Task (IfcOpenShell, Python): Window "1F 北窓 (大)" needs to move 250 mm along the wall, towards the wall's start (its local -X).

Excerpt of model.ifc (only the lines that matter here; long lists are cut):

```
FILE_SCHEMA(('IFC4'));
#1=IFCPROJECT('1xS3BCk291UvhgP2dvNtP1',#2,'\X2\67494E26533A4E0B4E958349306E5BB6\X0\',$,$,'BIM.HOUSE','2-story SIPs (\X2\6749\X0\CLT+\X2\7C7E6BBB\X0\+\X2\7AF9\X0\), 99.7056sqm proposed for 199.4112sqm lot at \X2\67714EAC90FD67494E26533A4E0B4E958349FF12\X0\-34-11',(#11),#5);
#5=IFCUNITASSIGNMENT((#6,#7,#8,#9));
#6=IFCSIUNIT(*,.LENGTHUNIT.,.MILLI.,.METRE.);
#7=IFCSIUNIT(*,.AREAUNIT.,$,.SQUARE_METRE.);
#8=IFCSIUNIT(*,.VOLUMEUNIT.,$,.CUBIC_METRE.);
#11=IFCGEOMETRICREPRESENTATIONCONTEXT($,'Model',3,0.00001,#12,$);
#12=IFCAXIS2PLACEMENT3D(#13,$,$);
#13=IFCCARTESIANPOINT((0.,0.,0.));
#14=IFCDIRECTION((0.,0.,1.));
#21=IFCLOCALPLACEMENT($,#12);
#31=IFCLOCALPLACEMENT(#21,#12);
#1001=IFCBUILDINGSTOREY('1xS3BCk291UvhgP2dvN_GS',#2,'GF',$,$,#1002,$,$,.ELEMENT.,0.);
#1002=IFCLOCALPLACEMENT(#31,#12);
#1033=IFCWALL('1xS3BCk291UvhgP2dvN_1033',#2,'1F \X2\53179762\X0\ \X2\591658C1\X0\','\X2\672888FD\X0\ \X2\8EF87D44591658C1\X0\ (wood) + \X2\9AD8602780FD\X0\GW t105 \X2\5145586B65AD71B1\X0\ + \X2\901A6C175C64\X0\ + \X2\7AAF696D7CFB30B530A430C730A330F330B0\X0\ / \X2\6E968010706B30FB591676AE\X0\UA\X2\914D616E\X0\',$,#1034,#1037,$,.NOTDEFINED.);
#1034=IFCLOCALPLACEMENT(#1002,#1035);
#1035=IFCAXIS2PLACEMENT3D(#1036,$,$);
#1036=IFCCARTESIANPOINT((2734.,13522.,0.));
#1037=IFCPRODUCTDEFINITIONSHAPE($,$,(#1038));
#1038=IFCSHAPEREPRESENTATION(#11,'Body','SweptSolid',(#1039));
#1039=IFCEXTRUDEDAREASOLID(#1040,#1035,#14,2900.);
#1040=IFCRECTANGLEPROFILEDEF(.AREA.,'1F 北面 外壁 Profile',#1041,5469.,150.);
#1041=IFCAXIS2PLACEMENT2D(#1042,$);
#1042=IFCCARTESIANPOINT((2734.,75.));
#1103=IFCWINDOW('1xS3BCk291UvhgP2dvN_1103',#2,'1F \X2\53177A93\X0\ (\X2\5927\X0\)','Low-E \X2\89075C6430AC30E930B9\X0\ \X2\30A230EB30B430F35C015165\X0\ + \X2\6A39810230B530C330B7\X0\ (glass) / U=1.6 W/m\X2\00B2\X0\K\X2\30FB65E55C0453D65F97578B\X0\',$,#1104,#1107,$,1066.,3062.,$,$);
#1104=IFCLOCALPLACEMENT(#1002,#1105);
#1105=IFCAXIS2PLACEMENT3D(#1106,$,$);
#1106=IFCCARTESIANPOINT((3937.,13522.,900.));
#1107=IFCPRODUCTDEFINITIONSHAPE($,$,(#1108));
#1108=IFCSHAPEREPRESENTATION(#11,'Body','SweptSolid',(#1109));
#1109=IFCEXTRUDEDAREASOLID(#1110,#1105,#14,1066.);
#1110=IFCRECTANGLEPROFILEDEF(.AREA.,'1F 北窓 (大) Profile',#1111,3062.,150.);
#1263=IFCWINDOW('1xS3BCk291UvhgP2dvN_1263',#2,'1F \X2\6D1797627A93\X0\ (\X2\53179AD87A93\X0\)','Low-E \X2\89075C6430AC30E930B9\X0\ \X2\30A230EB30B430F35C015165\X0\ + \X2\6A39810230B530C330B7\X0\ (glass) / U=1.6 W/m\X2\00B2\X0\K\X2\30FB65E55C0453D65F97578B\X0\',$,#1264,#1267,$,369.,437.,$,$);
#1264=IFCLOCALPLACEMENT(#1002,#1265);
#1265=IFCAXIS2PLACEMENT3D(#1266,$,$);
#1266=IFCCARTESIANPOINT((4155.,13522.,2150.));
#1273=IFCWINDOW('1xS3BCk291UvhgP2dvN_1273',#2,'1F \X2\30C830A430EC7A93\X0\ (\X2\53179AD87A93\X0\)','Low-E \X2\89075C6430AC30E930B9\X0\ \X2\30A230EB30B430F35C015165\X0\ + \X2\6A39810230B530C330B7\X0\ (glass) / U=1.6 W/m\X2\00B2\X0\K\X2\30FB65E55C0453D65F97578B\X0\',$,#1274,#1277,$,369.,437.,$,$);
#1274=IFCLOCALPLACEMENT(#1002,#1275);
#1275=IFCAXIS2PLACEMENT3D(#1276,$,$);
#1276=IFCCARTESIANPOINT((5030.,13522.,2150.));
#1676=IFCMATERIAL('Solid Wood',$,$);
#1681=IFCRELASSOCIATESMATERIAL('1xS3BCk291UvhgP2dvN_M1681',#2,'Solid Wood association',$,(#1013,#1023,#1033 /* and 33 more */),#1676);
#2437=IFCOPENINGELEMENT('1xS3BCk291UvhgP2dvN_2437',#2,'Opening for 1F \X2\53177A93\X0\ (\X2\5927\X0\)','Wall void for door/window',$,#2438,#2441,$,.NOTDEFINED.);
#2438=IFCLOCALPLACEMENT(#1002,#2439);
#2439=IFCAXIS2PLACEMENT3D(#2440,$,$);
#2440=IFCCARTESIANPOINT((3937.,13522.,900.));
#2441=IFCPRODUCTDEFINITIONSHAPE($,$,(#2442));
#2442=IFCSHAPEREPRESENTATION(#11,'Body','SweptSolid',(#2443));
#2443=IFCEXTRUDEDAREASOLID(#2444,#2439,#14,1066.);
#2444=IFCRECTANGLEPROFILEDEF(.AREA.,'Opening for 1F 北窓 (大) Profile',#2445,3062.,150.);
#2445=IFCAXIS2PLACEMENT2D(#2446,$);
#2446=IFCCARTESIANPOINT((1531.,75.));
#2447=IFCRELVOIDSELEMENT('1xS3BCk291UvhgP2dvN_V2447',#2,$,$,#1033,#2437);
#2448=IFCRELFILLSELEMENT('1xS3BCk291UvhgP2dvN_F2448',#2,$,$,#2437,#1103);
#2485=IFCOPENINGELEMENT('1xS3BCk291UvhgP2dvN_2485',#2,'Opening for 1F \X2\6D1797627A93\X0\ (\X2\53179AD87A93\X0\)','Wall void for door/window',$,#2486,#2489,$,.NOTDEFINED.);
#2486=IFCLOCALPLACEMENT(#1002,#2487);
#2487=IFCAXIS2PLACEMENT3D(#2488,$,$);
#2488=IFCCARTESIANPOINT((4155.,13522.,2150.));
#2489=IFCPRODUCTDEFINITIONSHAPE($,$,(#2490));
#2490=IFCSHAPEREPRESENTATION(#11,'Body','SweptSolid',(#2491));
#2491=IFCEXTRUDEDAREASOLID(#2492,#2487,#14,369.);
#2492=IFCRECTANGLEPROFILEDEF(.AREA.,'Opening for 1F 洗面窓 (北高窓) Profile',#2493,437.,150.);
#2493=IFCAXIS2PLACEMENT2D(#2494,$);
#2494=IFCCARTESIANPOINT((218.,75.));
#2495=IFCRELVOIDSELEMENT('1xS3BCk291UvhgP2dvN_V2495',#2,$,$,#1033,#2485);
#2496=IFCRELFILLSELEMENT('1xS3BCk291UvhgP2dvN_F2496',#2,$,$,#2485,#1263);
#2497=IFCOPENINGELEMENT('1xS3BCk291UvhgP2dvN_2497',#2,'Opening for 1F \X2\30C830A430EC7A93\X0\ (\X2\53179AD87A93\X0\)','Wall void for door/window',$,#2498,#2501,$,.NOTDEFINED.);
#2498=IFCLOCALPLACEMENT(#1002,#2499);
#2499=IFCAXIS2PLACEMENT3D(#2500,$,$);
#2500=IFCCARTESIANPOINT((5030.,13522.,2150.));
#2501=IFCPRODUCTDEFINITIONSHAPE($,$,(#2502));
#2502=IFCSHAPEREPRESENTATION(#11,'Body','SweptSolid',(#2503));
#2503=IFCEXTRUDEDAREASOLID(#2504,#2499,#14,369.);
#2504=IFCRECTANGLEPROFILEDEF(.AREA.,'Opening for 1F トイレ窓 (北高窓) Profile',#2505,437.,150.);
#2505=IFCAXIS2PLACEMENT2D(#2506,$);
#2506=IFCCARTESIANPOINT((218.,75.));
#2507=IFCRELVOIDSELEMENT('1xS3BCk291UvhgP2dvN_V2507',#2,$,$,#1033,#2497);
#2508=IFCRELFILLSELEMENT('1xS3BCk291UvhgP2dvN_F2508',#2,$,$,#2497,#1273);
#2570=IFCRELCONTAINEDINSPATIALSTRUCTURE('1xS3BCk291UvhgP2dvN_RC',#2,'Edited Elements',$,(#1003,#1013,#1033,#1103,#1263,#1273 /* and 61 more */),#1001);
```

```python
import ifcopenshell
import ifcopenshell.api.geometry
import ifcopenshell.util.placement
import ifcopenshell.util.unit

model = ifcopenshell.open("model.ifc")
unit_scale = ifcopenshell.util.unit.calculate_unit_scale(model)

window = model.by_guid("1xS3BCk291UvhgP2dvN_1103")
opening = window.FillsVoids[0].RelatingOpeningElement
wall = opening.VoidsElements[0].RelatingBuildingElement

wall_matrix = ifcopenshell.util.placement.get_local_placement(wall.ObjectPlacement)
shift = wall_matrix[:3, 0] * -0.25 / unit_scale
before = ifcopenshell.util.placement.get_local_placement(window.ObjectPlacement)[:3, 3].copy()

# The window is not placed relative to its opening, so move both.
for product in (opening, window):
    matrix = ifcopenshell.util.placement.get_local_placement(product.ObjectPlacement)
    matrix[:3, 3] += shift
    ifcopenshell.api.geometry.edit_object_placement(model, product=product, matrix=matrix, is_si=False)

after = ifcopenshell.util.placement.get_local_placement(window.ObjectPlacement)[:3, 3]
print("window moved by", (after - before).round(3) + 0.0)

model.write("model_v2.ifc")
```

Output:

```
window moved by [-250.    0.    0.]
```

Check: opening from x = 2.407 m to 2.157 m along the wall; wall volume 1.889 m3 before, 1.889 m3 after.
